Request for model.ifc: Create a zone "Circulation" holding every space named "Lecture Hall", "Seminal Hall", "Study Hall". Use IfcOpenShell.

First a look at what the model holds.

```python
import ifcopenshell

model = ifcopenshell.open("model.ifc")
print(model.schema)
seen = {}
for space in model.by_type("IfcSpace"):
    seen[space.LongName] = seen.get(space.LongName, 0) + 1
for name, count in sorted(seen.items(), key=str):
    print(count, "x", name)
print("zones:", [z.Name for z in model.by_type("IfcZone")][:20])
```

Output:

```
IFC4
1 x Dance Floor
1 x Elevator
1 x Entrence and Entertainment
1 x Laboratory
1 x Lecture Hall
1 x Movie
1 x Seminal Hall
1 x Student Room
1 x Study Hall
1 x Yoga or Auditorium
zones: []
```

```python
import ifcopenshell
import ifcopenshell.api.group
import ifcopenshell.api.root

model = ifcopenshell.open("model.ifc")

names = {"Lecture Hall", "Seminal Hall", "Study Hall"}
spaces = [s for s in model.by_type("IfcSpace") if s.LongName in names]

zone = ifcopenshell.api.root.create_entity(model, ifc_class="IfcZone", name="Circulation")
ifcopenshell.api.group.assign_group(model, products=spaces, group=zone)
print(len(spaces), "spaces in", zone.Name)

model.write("model_rev.ifc")
```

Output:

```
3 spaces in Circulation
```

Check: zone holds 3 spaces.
